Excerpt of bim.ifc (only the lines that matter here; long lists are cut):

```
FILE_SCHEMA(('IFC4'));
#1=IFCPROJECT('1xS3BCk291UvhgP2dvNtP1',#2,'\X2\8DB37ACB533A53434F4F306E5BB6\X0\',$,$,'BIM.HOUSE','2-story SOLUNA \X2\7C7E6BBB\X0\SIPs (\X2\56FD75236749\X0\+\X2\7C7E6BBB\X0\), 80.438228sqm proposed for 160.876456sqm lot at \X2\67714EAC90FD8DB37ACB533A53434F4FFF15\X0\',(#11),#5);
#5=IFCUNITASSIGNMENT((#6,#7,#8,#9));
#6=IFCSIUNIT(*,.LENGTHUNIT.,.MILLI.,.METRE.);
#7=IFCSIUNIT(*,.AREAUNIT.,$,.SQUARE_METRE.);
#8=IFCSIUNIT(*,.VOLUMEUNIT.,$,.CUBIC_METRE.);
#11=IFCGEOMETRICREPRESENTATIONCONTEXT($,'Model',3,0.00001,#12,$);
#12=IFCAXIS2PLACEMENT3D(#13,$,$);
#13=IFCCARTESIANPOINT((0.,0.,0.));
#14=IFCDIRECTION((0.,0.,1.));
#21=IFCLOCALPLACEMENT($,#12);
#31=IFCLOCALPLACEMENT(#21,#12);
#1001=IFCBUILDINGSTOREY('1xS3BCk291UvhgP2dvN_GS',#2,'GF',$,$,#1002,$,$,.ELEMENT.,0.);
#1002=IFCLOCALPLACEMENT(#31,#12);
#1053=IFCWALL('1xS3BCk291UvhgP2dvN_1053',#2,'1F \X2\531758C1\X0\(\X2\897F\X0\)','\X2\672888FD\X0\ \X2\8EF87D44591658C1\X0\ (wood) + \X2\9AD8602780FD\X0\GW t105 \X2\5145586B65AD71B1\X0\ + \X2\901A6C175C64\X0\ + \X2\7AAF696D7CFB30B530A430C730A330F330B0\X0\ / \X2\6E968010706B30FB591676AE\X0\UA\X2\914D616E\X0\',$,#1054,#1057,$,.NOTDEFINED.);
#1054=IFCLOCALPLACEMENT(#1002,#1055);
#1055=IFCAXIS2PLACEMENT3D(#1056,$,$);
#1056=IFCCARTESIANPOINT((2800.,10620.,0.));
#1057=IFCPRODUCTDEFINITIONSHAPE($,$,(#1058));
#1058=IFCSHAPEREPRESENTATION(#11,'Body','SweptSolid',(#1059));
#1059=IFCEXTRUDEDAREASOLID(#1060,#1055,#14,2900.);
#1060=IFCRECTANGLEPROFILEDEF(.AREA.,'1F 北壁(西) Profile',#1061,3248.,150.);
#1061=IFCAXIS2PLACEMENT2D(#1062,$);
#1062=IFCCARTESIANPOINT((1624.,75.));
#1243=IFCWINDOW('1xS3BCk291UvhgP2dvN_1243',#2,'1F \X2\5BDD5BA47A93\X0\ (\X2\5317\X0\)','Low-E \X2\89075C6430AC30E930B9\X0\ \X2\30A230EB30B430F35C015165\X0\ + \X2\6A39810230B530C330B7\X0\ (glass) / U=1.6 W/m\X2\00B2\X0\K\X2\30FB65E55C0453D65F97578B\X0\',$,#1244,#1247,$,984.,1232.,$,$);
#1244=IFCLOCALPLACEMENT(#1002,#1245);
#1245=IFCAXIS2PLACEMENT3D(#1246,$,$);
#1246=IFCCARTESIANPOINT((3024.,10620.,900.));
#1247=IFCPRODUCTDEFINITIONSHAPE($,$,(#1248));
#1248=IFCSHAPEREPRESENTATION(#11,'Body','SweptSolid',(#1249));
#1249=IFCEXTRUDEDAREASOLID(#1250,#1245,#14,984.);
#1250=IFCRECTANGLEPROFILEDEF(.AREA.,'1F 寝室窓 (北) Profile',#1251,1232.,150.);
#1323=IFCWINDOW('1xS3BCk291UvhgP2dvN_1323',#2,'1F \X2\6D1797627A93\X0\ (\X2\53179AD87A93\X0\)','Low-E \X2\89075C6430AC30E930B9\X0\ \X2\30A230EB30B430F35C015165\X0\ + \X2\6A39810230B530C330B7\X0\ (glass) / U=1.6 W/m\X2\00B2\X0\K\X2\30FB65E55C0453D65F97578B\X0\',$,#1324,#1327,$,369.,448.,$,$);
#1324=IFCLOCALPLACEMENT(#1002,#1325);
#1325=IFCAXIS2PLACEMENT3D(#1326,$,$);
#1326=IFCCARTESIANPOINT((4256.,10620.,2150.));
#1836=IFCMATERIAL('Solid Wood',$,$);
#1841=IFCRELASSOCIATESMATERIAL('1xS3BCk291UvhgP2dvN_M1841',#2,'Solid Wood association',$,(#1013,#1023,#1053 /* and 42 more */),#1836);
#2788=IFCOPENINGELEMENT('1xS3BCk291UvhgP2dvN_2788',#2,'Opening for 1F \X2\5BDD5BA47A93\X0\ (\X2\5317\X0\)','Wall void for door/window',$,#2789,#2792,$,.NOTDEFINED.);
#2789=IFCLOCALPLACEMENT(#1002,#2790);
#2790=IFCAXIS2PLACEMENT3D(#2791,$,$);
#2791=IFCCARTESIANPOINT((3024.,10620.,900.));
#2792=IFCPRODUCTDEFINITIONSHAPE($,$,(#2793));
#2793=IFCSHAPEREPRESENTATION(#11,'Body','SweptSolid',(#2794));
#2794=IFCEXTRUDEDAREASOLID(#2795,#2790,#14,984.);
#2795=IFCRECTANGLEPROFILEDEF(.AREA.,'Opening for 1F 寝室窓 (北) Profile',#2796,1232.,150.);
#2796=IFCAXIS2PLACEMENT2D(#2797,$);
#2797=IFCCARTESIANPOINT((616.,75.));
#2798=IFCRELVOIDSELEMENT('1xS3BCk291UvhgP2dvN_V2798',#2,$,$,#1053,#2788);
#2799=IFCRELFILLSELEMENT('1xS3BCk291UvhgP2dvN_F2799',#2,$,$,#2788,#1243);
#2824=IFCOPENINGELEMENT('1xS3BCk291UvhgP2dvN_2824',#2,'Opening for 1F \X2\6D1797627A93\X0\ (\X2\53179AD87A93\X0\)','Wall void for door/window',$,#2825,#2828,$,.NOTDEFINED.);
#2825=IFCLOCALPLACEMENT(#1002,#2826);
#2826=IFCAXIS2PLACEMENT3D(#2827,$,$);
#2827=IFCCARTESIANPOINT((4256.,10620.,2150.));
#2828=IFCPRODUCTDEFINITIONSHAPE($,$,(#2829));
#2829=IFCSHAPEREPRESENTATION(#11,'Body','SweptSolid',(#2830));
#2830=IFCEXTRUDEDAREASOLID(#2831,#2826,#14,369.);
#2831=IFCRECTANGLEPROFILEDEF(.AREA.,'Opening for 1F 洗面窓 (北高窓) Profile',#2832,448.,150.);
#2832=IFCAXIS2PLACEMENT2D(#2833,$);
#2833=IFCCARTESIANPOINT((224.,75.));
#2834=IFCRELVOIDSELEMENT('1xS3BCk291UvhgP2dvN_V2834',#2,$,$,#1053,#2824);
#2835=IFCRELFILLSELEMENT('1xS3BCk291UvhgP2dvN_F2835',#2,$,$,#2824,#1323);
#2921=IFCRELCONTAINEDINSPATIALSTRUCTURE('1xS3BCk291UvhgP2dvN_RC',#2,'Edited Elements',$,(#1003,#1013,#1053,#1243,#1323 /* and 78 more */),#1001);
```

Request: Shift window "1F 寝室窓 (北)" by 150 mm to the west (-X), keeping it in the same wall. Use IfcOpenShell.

```python
import ifcopenshell
import ifcopenshell.api.geometry
import ifcopenshell.util.placement
import ifcopenshell.util.unit

model = ifcopenshell.open("bim.ifc")
unit_scale = ifcopenshell.util.unit.calculate_unit_scale(model)

window = model.by_guid("1xS3BCk291UvhgP2dvN_1243")
opening = window.FillsVoids[0].RelatingOpeningElement
wall = opening.VoidsElements[0].RelatingBuildingElement

wall_matrix = ifcopenshell.util.placement.get_local_placement(wall.ObjectPlacement)
shift = wall_matrix[:3, 0] * -0.15 / unit_scale
before = ifcopenshell.util.placement.get_local_placement(window.ObjectPlacement)[:3, 3].copy()

# The window is not placed relative to its opening, so move both.
for product in (opening, window):
    matrix = ifcopenshell.util.placement.get_local_placement(product.ObjectPlacement)
    matrix[:3, 3] += shift
    ifcopenshell.api.geometry.edit_object_placement(model, product=product, matrix=matrix, is_si=False)

after = ifcopenshell.util.placement.get_local_placement(window.ObjectPlacement)[:3, 3]
print("window moved by", (after - before).round(3) + 0.0)

model.write("bim_edited.ifc")
```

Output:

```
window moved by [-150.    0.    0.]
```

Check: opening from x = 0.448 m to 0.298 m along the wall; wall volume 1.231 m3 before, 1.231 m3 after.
